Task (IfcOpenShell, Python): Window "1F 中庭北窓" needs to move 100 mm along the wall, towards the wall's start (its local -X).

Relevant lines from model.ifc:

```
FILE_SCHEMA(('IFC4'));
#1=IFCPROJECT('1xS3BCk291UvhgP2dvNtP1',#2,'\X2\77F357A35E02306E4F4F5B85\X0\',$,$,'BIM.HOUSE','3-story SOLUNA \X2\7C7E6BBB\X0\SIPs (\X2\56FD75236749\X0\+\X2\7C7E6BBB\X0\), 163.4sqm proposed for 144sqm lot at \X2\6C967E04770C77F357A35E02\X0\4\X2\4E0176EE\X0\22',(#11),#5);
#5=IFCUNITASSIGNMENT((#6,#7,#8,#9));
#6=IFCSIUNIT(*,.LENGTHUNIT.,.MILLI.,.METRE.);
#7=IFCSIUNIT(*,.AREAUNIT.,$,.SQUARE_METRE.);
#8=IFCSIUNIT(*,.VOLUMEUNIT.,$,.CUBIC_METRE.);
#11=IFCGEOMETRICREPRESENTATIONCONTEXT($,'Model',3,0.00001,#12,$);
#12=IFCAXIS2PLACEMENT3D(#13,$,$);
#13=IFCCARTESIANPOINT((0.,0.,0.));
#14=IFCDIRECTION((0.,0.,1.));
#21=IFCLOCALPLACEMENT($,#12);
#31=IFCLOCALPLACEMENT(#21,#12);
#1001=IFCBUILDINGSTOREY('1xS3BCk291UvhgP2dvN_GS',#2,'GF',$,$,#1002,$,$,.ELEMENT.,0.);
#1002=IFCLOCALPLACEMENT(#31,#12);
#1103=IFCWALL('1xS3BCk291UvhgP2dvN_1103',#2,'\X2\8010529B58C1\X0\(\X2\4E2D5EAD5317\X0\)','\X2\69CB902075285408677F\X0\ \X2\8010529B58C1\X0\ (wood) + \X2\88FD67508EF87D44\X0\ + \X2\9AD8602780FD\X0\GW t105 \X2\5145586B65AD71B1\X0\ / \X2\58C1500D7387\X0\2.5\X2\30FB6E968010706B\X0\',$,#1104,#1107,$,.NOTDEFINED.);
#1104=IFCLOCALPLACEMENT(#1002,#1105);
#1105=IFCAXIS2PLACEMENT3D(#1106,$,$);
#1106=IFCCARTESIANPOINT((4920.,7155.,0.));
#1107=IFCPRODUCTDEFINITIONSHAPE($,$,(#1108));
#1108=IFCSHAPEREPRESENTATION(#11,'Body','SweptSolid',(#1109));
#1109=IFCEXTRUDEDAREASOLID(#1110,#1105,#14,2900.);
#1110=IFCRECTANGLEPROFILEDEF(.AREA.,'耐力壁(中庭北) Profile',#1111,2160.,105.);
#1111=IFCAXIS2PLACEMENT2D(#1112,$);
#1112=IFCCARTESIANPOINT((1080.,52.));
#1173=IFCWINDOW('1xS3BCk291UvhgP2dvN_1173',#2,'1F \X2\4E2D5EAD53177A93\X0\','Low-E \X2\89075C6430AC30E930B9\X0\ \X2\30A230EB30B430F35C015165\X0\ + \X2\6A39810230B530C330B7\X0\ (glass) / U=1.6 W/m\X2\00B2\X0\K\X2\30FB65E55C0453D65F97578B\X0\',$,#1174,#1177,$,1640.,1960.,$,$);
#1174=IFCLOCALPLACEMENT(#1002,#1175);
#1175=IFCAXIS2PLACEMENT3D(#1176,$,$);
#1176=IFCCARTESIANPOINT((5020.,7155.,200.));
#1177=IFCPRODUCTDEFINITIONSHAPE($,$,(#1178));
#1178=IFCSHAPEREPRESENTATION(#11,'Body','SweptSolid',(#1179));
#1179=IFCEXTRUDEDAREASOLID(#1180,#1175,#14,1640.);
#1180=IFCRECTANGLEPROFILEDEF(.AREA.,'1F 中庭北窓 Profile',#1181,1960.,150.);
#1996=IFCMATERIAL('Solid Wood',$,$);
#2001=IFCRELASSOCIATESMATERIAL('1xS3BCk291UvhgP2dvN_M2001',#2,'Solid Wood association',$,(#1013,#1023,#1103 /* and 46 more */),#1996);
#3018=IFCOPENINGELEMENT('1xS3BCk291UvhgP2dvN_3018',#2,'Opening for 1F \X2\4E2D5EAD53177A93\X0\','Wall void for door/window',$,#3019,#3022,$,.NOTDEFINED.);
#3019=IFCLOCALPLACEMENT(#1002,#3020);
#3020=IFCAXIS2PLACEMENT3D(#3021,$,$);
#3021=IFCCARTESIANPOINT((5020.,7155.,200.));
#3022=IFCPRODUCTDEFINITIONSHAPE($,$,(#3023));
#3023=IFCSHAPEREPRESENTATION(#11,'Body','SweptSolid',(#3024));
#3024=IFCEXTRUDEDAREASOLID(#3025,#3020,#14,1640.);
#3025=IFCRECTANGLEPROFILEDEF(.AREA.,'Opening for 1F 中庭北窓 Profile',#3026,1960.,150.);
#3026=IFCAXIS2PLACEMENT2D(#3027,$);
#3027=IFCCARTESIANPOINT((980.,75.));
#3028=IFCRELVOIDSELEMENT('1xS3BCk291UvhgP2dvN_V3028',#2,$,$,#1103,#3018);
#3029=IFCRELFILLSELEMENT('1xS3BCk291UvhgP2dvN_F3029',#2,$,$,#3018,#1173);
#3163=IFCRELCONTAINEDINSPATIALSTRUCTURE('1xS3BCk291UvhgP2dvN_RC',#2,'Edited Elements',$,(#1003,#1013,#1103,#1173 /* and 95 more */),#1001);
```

```python
import ifcopenshell
import ifcopenshell.api.geometry
import ifcopenshell.util.placement
import ifcopenshell.util.unit

model = ifcopenshell.open("model.ifc")
unit_scale = ifcopenshell.util.unit.calculate_unit_scale(model)

window = model.by_guid("1xS3BCk291UvhgP2dvN_1173")
opening = window.FillsVoids[0].RelatingOpeningElement
wall = opening.VoidsElements[0].RelatingBuildingElement

wall_matrix = ifcopenshell.util.placement.get_local_placement(wall.ObjectPlacement)
shift = wall_matrix[:3, 0] * -0.1 / unit_scale
before = ifcopenshell.util.placement.get_local_placement(window.ObjectPlacement)[:3, 3].copy()

# The window is not placed relative to its opening, so move both.
for product in (opening, window):
    matrix = ifcopenshell.util.placement.get_local_placement(product.ObjectPlacement)
    matrix[:3, 3] += shift
    ifcopenshell.api.geometry.edit_object_placement(model, product=product, matrix=matrix, is_si=False)

after = ifcopenshell.util.placement.get_local_placement(window.ObjectPlacement)[:3, 3]
print("window moved by", (after - before).round(3) + 0.0)

model.write("model_updated.ifc")
```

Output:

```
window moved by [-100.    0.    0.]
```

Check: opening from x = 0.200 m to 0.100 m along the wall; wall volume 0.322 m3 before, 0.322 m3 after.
